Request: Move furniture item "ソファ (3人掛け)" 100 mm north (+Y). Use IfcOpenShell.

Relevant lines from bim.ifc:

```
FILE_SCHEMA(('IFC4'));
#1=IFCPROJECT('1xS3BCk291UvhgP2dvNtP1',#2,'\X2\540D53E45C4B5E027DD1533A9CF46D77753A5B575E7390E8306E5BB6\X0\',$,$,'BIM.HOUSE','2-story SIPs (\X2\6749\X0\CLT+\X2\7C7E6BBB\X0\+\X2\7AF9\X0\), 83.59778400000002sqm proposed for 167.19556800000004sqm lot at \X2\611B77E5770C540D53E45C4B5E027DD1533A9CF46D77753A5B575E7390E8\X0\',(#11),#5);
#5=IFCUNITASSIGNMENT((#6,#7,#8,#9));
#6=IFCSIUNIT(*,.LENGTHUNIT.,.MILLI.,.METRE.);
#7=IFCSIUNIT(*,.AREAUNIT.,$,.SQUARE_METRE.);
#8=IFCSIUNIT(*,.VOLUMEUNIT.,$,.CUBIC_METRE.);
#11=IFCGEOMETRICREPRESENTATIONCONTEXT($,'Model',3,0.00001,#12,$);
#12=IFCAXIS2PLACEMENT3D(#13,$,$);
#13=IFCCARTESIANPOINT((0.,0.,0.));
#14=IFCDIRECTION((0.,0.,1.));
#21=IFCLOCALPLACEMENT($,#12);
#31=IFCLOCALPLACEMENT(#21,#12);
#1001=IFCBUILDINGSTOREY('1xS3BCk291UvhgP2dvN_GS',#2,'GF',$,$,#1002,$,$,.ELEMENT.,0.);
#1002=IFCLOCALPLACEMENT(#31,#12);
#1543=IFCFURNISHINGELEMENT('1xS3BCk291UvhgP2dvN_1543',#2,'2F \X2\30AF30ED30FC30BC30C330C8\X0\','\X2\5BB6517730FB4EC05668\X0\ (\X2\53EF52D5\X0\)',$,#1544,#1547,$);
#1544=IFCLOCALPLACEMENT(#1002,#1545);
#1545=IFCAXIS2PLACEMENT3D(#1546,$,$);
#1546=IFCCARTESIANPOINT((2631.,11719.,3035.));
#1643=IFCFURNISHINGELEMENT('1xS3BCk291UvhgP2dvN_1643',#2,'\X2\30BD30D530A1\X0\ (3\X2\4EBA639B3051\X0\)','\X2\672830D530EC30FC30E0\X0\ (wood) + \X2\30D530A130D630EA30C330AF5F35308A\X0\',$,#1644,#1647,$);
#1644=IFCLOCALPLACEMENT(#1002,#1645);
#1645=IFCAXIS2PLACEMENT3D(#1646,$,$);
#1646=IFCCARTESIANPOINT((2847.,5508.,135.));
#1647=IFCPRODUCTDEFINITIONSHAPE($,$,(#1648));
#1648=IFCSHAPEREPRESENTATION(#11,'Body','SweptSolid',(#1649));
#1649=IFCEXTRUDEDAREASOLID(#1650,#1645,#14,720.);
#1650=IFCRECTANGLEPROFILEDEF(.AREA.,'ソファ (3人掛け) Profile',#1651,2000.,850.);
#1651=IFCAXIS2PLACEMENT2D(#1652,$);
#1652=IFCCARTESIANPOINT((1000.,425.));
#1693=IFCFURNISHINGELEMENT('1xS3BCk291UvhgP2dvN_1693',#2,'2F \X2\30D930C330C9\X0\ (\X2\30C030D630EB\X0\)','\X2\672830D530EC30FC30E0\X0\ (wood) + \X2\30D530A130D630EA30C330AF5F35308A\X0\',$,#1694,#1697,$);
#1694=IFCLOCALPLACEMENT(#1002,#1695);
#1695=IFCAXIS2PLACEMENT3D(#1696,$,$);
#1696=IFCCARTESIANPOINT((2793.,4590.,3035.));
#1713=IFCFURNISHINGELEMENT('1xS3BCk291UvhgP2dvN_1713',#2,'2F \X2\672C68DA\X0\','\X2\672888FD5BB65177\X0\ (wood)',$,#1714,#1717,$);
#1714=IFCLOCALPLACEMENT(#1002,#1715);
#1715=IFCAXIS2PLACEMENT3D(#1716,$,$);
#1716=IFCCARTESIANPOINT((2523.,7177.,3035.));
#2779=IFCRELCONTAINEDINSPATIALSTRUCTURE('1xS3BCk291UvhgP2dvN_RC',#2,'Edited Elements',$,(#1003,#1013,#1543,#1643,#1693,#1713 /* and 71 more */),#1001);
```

```python
import ifcopenshell
import ifcopenshell.api.geometry
import ifcopenshell.util.placement

model = ifcopenshell.open("bim.ifc")

item = model.by_id(1643)
matrix = ifcopenshell.util.placement.get_local_placement(item.ObjectPlacement)
matrix[1, 3] += 100.0
ifcopenshell.api.geometry.edit_object_placement(model, product=item, matrix=matrix, is_si=False)

print(ifcopenshell.util.placement.get_local_placement(item.ObjectPlacement).round(3) + 0.0)

model.write("bim_v2.ifc")
```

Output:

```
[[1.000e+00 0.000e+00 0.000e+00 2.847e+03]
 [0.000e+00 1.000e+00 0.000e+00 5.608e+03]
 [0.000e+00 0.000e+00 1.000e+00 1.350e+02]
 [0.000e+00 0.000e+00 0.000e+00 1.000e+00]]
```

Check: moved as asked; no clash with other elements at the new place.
